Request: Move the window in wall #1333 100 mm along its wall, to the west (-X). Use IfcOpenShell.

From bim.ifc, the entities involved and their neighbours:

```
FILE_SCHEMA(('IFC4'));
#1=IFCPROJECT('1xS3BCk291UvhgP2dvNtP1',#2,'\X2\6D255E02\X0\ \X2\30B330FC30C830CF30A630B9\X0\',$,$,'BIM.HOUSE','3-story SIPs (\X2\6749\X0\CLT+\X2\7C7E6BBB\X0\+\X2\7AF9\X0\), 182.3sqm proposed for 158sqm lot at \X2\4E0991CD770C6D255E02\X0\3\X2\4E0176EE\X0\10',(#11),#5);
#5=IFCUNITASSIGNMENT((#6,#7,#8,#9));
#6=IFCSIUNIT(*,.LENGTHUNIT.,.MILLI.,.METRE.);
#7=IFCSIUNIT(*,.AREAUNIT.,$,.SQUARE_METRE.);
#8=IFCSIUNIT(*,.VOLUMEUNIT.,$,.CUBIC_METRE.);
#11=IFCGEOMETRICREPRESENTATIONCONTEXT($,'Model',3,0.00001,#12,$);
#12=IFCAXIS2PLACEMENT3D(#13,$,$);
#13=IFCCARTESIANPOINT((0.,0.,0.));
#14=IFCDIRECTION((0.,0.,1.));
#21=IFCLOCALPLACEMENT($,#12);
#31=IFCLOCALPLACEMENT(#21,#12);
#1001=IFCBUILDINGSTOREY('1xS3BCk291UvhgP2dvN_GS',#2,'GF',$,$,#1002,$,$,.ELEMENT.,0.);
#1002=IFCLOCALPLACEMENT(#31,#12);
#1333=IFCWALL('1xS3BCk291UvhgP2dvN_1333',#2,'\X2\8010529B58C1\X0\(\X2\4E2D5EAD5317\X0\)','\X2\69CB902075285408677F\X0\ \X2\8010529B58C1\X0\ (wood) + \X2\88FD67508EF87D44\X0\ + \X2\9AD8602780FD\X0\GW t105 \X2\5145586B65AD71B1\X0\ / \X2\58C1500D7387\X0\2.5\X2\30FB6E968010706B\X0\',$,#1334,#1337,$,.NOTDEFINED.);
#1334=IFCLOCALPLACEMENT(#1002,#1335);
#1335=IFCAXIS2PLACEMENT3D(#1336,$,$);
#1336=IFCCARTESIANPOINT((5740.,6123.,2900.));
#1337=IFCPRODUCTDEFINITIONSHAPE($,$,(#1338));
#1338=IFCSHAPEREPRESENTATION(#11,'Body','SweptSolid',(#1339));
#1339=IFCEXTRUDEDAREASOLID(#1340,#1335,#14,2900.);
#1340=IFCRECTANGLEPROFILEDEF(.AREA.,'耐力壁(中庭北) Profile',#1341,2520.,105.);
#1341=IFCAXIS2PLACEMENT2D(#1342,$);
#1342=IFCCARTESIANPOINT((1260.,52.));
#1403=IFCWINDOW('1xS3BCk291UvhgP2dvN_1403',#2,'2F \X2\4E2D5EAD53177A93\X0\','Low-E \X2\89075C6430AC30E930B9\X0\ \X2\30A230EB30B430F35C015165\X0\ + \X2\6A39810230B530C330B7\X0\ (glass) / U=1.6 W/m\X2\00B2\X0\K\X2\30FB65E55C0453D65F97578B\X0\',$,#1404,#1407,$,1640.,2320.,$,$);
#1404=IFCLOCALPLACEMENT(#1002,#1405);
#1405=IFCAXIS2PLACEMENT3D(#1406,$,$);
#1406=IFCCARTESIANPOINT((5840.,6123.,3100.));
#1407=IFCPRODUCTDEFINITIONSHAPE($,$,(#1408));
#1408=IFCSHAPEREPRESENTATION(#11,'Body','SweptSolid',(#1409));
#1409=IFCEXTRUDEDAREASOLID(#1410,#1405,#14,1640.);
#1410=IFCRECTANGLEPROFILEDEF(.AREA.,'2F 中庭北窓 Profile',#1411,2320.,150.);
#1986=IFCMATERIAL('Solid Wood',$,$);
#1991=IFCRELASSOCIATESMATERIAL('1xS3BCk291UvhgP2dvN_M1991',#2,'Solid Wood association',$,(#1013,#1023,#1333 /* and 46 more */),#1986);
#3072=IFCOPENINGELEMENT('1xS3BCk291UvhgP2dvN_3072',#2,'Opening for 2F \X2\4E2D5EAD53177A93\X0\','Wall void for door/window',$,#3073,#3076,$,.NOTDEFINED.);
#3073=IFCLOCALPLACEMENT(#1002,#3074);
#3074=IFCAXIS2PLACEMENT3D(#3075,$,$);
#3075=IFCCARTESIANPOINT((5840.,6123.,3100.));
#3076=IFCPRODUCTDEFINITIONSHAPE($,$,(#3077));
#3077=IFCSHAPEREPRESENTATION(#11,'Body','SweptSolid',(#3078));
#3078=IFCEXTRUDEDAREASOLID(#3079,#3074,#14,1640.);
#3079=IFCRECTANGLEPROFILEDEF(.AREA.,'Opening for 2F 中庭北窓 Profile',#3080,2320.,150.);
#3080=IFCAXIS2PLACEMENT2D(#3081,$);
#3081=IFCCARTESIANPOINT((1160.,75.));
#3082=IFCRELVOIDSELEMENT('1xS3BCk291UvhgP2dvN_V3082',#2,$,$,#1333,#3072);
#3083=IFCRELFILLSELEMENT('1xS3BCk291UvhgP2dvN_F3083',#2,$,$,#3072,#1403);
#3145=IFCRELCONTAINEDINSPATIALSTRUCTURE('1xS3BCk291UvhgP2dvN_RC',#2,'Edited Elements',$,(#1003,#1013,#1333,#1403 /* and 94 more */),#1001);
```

```python
import ifcopenshell
import ifcopenshell.api.geometry
import ifcopenshell.util.placement

model = ifcopenshell.open("bim.ifc")

window = model.by_guid("1xS3BCk291UvhgP2dvN_1403")
opening = window.FillsVoids[0].RelatingOpeningElement
wall = opening.VoidsElements[0].RelatingBuildingElement

wall_matrix = ifcopenshell.util.placement.get_local_placement(wall.ObjectPlacement)
shift = wall_matrix[:3, 0] * -100.0
before = ifcopenshell.util.placement.get_local_placement(window.ObjectPlacement)[:3, 3].copy()

# The window is not placed relative to its opening, so move both.
for product in (opening, window):
    matrix = ifcopenshell.util.placement.get_local_placement(product.ObjectPlacement)
    matrix[:3, 3] += shift
    ifcopenshell.api.geometry.edit_object_placement(model, product=product, matrix=matrix, is_si=False)

after = ifcopenshell.util.placement.get_local_placement(window.ObjectPlacement)[:3, 3]
print("window moved by", (after - before).round(3) + 0.0)

model.write("bim_rev.ifc")
```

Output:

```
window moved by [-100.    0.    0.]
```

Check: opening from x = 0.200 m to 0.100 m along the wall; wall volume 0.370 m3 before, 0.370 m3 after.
